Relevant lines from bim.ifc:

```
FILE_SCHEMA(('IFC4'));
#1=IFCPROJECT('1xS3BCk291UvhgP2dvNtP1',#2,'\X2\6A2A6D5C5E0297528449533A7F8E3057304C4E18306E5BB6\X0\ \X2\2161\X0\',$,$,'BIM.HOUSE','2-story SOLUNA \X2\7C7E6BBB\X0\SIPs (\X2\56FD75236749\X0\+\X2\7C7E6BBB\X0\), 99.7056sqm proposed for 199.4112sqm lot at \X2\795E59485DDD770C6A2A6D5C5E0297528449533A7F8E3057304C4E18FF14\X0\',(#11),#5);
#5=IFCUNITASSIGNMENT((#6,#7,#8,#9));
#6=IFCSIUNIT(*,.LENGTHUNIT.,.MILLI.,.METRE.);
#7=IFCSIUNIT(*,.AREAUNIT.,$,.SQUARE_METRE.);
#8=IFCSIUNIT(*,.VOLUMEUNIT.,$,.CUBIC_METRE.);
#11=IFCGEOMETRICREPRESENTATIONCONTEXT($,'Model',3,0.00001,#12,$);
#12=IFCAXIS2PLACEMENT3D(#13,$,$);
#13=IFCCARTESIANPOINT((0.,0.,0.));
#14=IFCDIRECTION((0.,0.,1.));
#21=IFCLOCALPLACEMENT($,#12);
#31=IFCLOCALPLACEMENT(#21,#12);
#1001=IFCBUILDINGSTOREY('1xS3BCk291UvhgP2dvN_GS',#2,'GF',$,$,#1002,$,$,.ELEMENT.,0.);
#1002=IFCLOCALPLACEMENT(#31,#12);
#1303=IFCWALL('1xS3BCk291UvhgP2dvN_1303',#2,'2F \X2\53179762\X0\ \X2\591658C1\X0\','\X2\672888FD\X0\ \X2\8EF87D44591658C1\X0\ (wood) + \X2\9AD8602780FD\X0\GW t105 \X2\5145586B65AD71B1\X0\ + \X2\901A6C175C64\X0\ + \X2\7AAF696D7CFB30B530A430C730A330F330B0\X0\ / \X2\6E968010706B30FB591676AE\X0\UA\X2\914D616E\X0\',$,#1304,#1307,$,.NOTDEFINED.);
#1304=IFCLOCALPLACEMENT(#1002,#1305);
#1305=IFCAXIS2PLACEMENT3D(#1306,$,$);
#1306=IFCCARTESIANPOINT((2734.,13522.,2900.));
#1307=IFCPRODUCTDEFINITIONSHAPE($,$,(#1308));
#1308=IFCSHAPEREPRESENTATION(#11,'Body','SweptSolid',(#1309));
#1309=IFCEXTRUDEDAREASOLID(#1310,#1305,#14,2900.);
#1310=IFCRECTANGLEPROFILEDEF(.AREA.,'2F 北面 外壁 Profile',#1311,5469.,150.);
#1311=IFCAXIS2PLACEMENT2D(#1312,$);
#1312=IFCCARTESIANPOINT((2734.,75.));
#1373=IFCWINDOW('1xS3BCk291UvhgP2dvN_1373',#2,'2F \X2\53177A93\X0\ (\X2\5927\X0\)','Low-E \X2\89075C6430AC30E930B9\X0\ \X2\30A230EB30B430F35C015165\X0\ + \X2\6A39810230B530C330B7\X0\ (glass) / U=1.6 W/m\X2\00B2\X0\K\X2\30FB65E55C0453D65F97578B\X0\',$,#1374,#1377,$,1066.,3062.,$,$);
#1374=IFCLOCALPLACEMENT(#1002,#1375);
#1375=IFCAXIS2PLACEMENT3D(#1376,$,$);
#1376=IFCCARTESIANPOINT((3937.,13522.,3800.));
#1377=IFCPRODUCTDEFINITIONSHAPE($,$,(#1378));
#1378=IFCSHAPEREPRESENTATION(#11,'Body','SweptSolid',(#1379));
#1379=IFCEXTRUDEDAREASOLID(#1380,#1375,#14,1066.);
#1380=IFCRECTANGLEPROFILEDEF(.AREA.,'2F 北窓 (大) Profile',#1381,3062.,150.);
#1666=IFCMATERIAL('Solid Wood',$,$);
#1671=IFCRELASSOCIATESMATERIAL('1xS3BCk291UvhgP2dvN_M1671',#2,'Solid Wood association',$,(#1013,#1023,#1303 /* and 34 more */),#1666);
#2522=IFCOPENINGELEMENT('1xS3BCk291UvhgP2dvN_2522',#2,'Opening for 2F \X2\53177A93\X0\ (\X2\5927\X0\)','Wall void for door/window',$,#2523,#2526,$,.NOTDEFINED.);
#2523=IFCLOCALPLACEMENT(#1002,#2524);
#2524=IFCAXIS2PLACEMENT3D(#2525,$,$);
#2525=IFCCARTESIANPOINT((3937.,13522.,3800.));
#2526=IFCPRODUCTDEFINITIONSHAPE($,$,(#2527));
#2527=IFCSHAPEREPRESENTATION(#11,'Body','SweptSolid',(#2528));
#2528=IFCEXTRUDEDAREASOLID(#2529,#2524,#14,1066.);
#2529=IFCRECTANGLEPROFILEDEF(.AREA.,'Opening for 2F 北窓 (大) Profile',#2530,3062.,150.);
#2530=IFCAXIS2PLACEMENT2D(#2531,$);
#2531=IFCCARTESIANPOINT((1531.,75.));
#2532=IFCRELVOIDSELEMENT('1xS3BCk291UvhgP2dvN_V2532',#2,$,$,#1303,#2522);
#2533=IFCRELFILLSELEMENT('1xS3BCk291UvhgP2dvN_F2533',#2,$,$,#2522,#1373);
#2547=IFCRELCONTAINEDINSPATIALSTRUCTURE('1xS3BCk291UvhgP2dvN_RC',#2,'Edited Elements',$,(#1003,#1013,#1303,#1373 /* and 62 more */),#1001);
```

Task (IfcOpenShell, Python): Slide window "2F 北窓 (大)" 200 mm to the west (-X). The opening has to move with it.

```python
import ifcopenshell
import ifcopenshell.api.geometry
import ifcopenshell.util.placement
import ifcopenshell.util.unit

model = ifcopenshell.open("bim.ifc")
unit_scale = ifcopenshell.util.unit.calculate_unit_scale(model)

window = model.by_guid("1xS3BCk291UvhgP2dvN_1373")
opening = window.FillsVoids[0].RelatingOpeningElement
wall = opening.VoidsElements[0].RelatingBuildingElement

wall_matrix = ifcopenshell.util.placement.get_local_placement(wall.ObjectPlacement)
shift = wall_matrix[:3, 0] * -0.2 / unit_scale
before = ifcopenshell.util.placement.get_local_placement(window.ObjectPlacement)[:3, 3].copy()

# The window is not placed relative to its opening, so move both.
for product in (opening, window):
    matrix = ifcopenshell.util.placement.get_local_placement(product.ObjectPlacement)
    matrix[:3, 3] += shift
    ifcopenshell.api.geometry.edit_object_placement(model, product=product, matrix=matrix, is_si=False)

after = ifcopenshell.util.placement.get_local_placement(window.ObjectPlacement)[:3, 3]
print("window moved by", (after - before).round(3) + 0.0)

model.write("bim_updated.ifc")
```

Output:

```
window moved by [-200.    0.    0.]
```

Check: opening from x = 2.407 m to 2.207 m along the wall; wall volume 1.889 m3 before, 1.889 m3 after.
